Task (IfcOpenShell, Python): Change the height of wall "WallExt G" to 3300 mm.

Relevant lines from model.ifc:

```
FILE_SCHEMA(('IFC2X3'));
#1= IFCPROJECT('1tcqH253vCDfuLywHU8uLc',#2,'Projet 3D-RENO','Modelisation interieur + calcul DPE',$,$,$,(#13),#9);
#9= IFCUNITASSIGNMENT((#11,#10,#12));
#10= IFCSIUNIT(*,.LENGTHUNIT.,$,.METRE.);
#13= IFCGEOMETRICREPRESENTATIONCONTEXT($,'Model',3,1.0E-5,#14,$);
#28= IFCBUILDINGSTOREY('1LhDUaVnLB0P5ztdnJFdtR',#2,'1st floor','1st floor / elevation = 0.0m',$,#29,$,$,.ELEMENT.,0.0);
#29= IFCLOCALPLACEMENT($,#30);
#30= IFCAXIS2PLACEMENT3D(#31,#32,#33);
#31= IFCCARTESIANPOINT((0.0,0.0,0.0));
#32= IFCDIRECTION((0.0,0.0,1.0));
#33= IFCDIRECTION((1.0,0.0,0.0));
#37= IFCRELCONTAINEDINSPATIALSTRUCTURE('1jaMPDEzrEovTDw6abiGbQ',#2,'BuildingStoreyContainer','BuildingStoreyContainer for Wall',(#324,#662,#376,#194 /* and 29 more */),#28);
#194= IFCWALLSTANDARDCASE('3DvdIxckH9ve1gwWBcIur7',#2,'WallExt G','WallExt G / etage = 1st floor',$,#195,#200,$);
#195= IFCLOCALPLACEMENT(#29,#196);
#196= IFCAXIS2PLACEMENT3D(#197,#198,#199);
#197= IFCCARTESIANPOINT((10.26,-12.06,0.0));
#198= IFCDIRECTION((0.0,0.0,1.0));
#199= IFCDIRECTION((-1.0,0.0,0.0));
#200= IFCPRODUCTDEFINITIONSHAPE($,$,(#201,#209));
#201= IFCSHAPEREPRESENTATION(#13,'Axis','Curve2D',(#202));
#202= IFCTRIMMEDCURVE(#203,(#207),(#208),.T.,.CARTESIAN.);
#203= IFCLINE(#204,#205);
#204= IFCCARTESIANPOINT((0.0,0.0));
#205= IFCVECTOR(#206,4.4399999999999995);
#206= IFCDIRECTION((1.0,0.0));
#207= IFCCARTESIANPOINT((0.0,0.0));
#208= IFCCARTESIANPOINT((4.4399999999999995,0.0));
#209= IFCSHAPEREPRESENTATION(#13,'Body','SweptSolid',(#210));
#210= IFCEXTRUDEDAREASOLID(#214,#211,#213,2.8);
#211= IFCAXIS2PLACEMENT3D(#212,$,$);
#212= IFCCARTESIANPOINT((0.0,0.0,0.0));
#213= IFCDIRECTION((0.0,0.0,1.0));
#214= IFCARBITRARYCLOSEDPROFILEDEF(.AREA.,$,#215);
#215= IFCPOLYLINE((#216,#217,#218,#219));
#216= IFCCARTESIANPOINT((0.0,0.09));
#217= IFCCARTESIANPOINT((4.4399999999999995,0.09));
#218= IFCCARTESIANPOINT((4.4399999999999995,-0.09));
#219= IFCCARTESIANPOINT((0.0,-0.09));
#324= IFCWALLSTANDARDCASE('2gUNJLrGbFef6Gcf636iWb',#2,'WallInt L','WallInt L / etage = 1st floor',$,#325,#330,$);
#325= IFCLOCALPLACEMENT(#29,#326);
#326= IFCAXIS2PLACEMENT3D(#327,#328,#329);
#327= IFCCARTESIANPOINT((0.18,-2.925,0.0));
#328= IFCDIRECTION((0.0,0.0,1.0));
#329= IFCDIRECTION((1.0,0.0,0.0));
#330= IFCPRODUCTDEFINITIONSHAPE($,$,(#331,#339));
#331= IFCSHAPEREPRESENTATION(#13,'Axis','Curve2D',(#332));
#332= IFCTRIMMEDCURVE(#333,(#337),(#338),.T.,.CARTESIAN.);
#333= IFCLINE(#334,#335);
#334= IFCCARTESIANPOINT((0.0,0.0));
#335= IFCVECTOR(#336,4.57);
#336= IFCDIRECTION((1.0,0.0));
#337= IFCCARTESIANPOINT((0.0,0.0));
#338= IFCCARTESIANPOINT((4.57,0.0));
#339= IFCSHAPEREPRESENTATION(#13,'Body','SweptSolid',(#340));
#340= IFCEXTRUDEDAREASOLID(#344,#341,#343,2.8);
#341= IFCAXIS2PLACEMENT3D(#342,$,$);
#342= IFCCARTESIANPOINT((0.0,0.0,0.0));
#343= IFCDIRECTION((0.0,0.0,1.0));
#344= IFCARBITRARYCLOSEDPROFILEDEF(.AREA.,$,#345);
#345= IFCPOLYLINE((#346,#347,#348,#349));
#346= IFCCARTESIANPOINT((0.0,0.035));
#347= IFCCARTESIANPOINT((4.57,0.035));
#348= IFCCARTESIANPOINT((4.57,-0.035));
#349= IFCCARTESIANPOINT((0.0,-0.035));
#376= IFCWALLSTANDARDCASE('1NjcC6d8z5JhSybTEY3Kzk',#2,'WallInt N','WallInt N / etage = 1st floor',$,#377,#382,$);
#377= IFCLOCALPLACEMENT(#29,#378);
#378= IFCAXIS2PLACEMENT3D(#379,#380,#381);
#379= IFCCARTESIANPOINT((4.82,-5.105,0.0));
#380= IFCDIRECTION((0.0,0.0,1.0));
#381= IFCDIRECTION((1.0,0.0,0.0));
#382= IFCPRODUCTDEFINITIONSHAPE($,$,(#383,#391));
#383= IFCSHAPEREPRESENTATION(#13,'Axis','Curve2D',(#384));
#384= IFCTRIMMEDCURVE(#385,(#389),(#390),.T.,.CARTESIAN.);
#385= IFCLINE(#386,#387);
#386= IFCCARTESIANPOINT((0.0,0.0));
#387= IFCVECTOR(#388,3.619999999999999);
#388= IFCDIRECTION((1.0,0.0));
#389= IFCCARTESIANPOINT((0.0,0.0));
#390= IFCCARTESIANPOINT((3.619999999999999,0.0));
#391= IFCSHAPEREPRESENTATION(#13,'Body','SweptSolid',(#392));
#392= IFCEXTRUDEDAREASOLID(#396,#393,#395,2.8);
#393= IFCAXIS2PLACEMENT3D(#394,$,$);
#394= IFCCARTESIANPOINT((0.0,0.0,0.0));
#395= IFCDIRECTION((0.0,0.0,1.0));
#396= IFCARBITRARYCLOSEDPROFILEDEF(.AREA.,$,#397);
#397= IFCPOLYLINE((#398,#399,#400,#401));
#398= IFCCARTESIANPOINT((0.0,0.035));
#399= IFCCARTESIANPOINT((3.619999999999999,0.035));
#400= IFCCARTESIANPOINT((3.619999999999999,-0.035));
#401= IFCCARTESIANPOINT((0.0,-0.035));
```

```python
import ifcopenshell
import ifcopenshell.geom
import ifcopenshell.util.shape
import ifcopenshell.util.unit

model = ifcopenshell.open("model.ifc")
unit_scale = ifcopenshell.util.unit.calculate_unit_scale(model)
settings = ifcopenshell.geom.settings()


def volume(element):
    """Net volume in cubic metres, openings subtracted."""
    shape = ifcopenshell.geom.create_shape(settings, element)
    return ifcopenshell.util.shape.get_volume(shape.geometry)


wall = model.by_guid("3DvdIxckH9ve1gwWBcIur7")
before = volume(wall)

body = next(r for r in wall.Representation.Representations if r.RepresentationIdentifier == "Body")
solid = body.Items[0]
old_height = solid.Depth
solid.Depth = 3.3 / unit_scale
after = volume(wall)

print(f"height {old_height:g} -> {solid.Depth:g}, volume {before:.3f} -> {after:.3f} m3")

model.write("model_v2.ifc")
```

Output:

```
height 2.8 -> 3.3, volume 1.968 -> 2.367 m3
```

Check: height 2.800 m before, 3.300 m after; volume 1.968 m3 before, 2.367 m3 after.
